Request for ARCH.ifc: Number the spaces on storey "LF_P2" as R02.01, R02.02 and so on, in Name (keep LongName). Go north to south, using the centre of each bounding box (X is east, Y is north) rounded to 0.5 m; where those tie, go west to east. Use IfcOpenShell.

First a look at what the model holds.

```python
import ifcopenshell
import ifcopenshell.util.element
import ifcopenshell.util.placement

model = ifcopenshell.open("ARCH.ifc")
print(model.schema)
storey = next(s for s in model.by_type("IfcBuildingStorey") if s.Name == "LF_P2")
spaces = [e for e in ifcopenshell.util.element.get_decomposition(storey) if e.is_a("IfcSpace")]
for e in sorted(spaces, key=lambda e: e.id()):
    origin = ifcopenshell.util.placement.get_local_placement(e.ObjectPlacement)[:3, 3]
    print(e.id(), e.Name, e.LongName, origin.round(2) + 0.0, sep=" | ")
```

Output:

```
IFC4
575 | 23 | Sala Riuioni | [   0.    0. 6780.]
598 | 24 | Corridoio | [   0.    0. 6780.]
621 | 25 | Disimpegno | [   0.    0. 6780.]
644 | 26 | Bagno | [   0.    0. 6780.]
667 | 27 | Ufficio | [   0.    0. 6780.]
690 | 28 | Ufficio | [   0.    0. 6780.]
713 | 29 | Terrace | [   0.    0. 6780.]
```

```python
import ifcopenshell
import ifcopenshell.geom
import ifcopenshell.util.element
import ifcopenshell.util.shape

model = ifcopenshell.open("ARCH.ifc")
settings = ifcopenshell.geom.settings()
settings.set("use-world-coords", True)


def centre(element):
    shape = ifcopenshell.geom.create_shape(settings, element)
    return ifcopenshell.util.shape.get_bbox_centroid(shape.geometry)


storey = next(s for s in model.by_type("IfcBuildingStorey") if s.Name == "LF_P2")
spaces = [e for e in ifcopenshell.util.element.get_decomposition(storey) if e.is_a("IfcSpace")]

# Insertion points can sit at a corner or the storey origin, so sort by the geometry (in metres).
centres = {e: centre(e) for e in spaces}
spaces.sort(key=lambda e: (-round(centres[e][1] / 0.5), centres[e][0]))

for i, e in enumerate(spaces, start=1):
    number = f"R02.{i:02d}"
    e.Name = number
    print(e.id(), number)

model.write("ARCH_rev.ifc")
```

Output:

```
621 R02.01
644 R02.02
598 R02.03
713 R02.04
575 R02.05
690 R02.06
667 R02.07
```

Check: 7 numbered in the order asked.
